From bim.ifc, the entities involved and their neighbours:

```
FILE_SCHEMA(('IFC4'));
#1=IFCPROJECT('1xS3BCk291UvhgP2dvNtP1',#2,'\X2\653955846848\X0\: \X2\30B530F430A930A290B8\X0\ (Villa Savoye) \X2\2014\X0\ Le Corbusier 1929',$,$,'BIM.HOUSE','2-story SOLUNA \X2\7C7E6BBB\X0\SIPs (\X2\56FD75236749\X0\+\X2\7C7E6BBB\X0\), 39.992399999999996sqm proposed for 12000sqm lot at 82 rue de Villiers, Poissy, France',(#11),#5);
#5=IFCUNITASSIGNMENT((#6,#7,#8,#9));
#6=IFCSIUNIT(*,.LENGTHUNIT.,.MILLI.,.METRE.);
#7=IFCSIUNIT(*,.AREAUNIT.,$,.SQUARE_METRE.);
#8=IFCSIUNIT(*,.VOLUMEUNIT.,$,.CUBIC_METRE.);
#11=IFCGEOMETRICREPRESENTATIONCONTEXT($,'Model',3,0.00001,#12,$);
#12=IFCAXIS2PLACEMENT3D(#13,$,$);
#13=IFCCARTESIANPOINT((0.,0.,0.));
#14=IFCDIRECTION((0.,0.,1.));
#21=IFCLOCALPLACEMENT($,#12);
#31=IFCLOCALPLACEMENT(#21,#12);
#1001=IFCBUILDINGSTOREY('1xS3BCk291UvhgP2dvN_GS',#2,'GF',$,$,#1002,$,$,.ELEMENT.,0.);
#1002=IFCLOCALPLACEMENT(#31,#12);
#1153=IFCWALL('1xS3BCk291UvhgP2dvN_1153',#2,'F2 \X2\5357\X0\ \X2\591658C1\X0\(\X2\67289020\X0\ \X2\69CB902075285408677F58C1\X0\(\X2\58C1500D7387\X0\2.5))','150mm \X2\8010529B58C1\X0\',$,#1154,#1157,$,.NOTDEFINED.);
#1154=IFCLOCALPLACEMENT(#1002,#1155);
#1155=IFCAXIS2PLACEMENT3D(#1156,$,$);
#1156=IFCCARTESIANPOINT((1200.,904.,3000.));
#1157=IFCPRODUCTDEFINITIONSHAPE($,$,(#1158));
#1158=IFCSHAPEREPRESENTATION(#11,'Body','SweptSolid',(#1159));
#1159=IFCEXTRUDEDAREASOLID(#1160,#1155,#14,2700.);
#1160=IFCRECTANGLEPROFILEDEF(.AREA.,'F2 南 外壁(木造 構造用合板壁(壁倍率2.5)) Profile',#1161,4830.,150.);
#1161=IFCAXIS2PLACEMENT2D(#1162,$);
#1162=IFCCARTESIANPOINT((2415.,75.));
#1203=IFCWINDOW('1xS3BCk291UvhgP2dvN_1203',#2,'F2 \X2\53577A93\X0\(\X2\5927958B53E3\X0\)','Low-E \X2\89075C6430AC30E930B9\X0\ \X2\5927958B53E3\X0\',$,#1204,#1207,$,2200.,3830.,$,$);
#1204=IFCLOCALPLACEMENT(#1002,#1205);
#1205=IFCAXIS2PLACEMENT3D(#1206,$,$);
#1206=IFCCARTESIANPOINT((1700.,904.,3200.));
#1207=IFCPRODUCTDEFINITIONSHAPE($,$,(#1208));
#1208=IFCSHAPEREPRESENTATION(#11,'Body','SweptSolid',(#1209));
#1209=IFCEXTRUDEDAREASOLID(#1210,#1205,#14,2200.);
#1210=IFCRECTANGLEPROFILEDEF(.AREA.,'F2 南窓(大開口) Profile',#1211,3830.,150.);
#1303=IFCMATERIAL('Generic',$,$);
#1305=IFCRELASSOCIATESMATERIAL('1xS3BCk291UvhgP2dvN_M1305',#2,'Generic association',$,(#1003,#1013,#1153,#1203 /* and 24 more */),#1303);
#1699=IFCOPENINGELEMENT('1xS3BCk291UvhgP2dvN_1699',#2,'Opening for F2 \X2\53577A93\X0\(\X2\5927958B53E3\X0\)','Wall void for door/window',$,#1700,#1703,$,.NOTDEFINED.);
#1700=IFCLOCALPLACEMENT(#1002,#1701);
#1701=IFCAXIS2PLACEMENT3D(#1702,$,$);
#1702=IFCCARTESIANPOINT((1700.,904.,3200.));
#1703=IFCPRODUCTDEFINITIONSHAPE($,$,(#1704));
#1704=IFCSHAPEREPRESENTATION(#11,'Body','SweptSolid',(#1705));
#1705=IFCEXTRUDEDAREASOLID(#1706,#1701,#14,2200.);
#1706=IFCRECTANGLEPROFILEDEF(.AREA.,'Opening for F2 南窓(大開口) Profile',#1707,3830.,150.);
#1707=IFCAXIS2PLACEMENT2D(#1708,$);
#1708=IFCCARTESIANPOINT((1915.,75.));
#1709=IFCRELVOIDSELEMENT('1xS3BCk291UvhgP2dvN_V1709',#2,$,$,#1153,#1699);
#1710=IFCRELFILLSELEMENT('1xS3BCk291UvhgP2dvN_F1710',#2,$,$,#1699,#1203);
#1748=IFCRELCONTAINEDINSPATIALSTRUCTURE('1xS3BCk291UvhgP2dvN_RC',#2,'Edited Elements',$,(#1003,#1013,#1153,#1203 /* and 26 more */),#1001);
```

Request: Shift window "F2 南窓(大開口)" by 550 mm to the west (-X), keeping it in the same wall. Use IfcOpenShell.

```python
import ifcopenshell
import ifcopenshell.api.geometry
import ifcopenshell.util.placement
import ifcopenshell.util.unit

model = ifcopenshell.open("bim.ifc")
unit_scale = ifcopenshell.util.unit.calculate_unit_scale(model)

window = model.by_id(1203)
opening = window.FillsVoids[0].RelatingOpeningElement
wall = opening.VoidsElements[0].RelatingBuildingElement

wall_matrix = ifcopenshell.util.placement.get_local_placement(wall.ObjectPlacement)
shift = wall_matrix[:3, 0] * -0.55 / unit_scale
before = ifcopenshell.util.placement.get_local_placement(window.ObjectPlacement)[:3, 3].copy()

# The window is not placed relative to its opening, so move both.
for product in (opening, window):
    matrix = ifcopenshell.util.placement.get_local_placement(product.ObjectPlacement)
    matrix[:3, 3] += shift
    ifcopenshell.api.geometry.edit_object_placement(model, product=product, matrix=matrix, is_si=False)

after = ifcopenshell.util.placement.get_local_placement(window.ObjectPlacement)[:3, 3]
print("window moved by", (after - before).round(3) + 0.0)

model.write("bim_rev.ifc")
```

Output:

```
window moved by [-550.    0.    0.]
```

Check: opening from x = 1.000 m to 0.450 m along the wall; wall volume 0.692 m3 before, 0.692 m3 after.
